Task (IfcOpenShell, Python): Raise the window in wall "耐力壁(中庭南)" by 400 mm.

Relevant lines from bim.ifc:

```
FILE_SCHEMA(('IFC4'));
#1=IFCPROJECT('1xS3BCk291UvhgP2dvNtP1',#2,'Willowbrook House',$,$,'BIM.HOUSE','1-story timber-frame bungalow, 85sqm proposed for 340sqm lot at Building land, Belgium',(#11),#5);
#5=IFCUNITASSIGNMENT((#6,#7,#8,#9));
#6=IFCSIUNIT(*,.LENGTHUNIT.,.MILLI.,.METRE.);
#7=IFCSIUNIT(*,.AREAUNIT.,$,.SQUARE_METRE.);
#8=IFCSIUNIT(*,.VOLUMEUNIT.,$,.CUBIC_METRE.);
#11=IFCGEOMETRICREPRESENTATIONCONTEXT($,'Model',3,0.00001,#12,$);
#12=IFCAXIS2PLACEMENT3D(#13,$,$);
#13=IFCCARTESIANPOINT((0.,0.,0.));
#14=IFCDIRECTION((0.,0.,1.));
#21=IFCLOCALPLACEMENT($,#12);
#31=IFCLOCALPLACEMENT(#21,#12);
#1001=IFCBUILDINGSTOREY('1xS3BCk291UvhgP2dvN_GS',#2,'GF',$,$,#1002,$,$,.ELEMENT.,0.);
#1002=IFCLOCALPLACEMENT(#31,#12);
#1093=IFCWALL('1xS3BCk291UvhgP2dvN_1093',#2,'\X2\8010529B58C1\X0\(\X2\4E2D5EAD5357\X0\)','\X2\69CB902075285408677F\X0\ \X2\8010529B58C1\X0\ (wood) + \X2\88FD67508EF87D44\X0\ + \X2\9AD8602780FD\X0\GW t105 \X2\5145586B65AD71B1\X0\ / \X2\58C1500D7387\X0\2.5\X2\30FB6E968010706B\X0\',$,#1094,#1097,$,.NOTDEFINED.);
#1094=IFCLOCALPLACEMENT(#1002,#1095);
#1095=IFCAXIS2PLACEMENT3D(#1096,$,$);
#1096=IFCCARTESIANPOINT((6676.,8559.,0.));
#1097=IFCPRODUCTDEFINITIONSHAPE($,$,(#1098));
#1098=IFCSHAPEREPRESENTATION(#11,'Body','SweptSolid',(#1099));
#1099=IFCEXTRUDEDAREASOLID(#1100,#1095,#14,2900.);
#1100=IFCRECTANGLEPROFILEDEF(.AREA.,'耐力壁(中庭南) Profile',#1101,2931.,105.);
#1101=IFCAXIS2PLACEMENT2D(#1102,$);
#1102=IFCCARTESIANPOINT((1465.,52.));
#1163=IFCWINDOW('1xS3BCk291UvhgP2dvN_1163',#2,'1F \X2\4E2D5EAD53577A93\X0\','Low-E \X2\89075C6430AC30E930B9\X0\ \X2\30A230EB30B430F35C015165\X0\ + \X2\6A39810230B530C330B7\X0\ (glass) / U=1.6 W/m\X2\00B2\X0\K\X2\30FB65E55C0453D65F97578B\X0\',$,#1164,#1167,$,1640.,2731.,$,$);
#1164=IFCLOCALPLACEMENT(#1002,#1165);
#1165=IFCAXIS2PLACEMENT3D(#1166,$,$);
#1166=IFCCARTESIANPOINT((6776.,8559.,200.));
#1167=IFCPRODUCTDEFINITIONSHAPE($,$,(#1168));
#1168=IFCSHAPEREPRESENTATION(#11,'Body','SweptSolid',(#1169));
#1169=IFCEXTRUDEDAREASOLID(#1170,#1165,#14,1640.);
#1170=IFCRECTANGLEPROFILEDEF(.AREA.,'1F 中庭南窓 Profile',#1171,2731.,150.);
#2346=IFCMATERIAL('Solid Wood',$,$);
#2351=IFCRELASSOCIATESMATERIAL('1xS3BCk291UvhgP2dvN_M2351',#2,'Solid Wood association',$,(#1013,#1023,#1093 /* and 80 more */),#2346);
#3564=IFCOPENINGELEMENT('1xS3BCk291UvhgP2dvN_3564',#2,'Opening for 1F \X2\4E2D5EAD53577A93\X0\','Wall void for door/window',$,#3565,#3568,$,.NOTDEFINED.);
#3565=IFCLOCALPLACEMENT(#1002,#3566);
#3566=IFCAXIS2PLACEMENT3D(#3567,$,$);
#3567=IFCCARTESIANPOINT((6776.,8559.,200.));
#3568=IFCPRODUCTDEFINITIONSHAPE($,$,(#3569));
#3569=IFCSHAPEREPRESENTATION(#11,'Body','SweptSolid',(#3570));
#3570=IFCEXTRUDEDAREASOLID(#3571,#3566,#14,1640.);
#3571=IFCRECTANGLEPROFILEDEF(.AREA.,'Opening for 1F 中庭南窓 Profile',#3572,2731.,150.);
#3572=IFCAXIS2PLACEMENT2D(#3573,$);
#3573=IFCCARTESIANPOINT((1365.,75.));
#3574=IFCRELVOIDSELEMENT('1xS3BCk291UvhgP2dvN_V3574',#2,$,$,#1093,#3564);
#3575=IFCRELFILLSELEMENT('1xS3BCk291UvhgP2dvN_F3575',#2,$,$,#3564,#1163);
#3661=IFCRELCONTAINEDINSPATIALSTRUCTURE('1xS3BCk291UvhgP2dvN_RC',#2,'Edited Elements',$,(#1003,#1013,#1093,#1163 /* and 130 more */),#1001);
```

```python
import numpy as np
import ifcopenshell
import ifcopenshell.api.geometry
import ifcopenshell.util.placement
import ifcopenshell.util.unit

model = ifcopenshell.open("bim.ifc")
unit_scale = ifcopenshell.util.unit.calculate_unit_scale(model)

window = model.by_id(1163)
opening = window.FillsVoids[0].RelatingOpeningElement
dz = 0.4 / unit_scale

shift = np.array([0.0, 0.0, dz])
# The window is not placed relative to its opening, so move both.
for product in (opening, window):
    matrix = ifcopenshell.util.placement.get_local_placement(product.ObjectPlacement)
    matrix[:3, 3] += shift
    ifcopenshell.api.geometry.edit_object_placement(model, product=product, matrix=matrix, is_si=False)

print(f"moved by {dz * unit_scale:+.3f} m")

model.write("bim_rev.ifc")
```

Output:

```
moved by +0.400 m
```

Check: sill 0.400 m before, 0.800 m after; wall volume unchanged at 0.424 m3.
